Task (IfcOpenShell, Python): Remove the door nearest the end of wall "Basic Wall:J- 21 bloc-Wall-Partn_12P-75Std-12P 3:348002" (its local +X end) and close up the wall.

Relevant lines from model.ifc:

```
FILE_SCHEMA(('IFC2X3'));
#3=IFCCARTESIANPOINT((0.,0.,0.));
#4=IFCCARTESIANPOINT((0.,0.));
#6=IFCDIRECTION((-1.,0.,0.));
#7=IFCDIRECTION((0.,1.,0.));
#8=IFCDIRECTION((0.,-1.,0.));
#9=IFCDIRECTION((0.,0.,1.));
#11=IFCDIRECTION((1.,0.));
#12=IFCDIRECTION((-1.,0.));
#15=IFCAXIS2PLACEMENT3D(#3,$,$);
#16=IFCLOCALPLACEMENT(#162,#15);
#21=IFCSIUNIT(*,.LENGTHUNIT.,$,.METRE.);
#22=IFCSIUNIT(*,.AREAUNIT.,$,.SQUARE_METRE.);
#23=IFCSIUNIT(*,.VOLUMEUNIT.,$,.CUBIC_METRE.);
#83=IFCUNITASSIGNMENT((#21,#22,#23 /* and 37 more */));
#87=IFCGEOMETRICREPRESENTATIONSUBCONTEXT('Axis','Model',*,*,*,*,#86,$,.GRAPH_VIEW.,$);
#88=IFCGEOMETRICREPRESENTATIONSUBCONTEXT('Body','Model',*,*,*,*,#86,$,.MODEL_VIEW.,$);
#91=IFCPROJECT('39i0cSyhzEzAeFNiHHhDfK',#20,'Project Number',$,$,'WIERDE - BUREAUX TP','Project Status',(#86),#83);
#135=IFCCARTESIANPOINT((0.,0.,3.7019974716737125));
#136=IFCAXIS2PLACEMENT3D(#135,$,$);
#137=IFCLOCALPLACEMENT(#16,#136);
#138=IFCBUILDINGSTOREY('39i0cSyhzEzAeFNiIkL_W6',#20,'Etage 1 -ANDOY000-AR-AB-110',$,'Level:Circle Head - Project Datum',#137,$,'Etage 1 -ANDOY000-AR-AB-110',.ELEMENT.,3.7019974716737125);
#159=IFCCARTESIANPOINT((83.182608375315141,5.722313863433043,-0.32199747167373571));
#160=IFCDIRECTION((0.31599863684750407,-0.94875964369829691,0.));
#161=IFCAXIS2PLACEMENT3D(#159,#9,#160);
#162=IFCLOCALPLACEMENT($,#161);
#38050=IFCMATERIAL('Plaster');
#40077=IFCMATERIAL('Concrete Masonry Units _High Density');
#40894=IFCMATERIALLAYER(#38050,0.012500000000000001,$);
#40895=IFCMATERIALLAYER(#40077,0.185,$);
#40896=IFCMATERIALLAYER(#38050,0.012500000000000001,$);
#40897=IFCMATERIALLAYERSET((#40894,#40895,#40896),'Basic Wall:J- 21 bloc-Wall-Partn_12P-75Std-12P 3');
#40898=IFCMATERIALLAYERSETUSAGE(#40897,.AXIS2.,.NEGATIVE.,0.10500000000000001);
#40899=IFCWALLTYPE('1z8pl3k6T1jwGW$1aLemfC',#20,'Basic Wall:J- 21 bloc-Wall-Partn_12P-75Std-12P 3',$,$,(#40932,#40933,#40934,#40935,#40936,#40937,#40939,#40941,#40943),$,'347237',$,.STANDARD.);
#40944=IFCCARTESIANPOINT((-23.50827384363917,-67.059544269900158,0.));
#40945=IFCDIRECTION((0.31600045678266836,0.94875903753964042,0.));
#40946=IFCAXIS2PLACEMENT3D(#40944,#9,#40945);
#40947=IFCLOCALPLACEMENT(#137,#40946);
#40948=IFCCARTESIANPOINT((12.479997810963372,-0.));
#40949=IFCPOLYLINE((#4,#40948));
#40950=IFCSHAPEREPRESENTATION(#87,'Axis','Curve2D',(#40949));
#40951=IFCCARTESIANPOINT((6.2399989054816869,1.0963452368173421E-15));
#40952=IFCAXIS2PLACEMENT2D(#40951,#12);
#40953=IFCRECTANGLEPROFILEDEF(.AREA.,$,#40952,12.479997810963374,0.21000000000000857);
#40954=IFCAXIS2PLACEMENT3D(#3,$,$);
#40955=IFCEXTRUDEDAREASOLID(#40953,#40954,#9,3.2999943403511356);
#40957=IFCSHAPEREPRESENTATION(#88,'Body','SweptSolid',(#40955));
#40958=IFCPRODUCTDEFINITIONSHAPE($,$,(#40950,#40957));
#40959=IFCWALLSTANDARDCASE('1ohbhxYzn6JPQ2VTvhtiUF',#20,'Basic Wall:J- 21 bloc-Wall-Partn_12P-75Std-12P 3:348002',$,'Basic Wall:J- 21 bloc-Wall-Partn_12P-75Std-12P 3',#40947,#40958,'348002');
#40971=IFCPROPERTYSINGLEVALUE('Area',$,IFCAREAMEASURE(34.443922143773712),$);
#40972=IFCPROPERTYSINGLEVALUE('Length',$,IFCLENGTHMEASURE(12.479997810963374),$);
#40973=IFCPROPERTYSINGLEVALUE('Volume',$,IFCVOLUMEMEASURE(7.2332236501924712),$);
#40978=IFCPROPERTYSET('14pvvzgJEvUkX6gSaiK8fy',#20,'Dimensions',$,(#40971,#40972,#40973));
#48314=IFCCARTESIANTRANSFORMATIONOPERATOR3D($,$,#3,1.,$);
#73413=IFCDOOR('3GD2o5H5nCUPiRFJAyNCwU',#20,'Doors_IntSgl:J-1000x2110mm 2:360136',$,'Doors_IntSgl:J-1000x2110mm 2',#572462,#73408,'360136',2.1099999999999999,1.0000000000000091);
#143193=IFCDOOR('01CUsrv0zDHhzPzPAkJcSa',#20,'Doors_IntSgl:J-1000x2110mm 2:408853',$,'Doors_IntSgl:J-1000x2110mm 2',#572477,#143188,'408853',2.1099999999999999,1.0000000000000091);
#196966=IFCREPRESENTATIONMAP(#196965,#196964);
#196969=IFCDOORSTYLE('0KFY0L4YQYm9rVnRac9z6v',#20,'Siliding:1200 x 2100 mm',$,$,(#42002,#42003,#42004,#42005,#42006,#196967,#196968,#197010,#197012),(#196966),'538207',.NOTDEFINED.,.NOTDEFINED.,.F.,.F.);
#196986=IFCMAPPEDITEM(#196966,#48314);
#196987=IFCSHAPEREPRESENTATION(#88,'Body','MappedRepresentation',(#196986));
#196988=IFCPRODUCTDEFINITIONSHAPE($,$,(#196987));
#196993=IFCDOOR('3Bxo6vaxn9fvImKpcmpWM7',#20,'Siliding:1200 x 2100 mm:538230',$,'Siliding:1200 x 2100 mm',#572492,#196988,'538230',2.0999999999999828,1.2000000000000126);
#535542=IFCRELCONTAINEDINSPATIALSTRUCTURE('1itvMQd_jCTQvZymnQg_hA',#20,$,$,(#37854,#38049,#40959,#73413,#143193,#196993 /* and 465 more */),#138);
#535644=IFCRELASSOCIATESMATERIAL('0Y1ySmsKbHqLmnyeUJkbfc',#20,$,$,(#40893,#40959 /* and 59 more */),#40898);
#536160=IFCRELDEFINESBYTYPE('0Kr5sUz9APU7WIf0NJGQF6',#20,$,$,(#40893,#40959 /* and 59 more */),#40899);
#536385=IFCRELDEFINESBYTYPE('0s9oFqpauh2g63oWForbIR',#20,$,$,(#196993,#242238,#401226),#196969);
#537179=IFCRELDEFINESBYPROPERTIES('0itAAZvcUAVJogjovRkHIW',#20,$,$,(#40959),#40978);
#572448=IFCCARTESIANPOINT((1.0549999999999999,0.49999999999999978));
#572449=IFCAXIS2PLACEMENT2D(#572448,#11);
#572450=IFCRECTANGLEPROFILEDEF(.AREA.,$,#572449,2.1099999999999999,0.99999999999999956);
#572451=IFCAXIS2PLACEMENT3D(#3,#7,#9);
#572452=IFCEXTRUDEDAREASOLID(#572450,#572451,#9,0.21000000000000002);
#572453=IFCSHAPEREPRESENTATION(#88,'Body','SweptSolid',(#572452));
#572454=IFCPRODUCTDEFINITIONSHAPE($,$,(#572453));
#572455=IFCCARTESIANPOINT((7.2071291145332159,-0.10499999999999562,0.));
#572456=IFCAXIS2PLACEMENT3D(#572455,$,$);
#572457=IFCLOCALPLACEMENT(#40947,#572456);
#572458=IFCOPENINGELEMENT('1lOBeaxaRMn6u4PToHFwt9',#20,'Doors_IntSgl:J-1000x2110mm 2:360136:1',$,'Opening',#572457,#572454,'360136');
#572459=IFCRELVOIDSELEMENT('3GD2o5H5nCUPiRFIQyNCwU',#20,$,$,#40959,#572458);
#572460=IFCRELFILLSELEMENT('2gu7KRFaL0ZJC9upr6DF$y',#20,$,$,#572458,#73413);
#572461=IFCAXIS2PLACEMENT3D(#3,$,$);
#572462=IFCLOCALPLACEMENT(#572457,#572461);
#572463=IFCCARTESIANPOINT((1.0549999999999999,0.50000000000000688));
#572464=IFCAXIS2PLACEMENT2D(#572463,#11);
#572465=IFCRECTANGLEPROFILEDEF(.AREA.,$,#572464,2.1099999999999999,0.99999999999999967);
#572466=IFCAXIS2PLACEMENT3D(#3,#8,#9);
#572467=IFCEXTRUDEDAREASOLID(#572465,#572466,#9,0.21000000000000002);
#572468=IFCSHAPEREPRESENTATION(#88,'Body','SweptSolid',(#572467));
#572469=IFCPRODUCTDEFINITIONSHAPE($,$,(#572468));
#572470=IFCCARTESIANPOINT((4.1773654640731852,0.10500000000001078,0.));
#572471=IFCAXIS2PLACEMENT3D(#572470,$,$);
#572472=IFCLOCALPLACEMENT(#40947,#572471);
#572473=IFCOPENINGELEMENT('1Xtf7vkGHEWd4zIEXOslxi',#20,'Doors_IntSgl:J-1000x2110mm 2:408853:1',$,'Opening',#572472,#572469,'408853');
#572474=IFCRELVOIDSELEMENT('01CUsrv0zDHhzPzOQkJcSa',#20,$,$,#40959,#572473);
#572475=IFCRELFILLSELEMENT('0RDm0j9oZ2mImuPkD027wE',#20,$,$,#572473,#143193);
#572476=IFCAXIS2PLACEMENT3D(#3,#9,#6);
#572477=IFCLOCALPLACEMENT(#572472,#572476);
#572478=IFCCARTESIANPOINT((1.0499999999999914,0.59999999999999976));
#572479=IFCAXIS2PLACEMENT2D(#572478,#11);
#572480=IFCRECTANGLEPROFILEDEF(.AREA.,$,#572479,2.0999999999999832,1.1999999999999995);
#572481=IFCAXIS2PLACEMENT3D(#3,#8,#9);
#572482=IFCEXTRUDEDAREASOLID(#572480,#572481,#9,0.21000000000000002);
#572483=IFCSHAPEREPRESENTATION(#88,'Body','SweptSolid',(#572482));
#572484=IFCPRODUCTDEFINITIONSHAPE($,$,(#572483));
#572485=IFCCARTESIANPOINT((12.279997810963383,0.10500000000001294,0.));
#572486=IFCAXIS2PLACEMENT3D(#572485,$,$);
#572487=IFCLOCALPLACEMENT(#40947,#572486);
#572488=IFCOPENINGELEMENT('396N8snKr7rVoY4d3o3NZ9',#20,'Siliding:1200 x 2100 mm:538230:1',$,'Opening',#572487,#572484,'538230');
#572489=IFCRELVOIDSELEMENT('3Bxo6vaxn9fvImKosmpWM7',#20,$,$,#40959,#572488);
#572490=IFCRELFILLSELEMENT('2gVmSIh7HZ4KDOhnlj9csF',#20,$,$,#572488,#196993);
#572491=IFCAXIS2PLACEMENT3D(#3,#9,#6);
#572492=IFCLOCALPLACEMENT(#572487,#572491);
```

```python
import ifcopenshell
import ifcopenshell.api.feature
import ifcopenshell.api.pset
import ifcopenshell.api.root
import ifcopenshell.geom
import ifcopenshell.util.element
import ifcopenshell.util.shape
import ifcopenshell.util.unit

model = ifcopenshell.open("model.ifc")
area_scale = ifcopenshell.util.unit.calculate_unit_scale(model, "AREAUNIT")
volume_scale = ifcopenshell.util.unit.calculate_unit_scale(model, "VOLUMEUNIT")
settings = ifcopenshell.geom.settings()


def volume(element):
    """Net volume in cubic metres, openings subtracted."""
    shape = ifcopenshell.geom.create_shape(settings, element)
    return ifcopenshell.util.shape.get_volume(shape.geometry)


door = model.by_guid("3Bxo6vaxn9fvImKpcmpWM7")
opening = door.FillsVoids[0].RelatingOpeningElement
wall = opening.VoidsElements[0].RelatingBuildingElement
before = volume(wall)

ifcopenshell.api.root.remove_product(model, product=door)
ifcopenshell.api.feature.remove_feature(model, feature=opening)

after = volume(wall)
thickness = 0.21  # wall thickness in metres

# Update the wall's stored quantities.
pset = model.by_id(ifcopenshell.util.element.get_pset(wall, "Dimensions", should_inherit=False)["id"])
ifcopenshell.api.pset.edit_pset(model, pset=pset, properties={
    "Area": model.create_entity("IfcAreaMeasure", after / thickness / area_scale),
    "Volume": model.create_entity("IfcVolumeMeasure", after / volume_scale),
})

print(f"wall volume {before:.3f} -> {after:.3f} m3")

model.write("model_updated.ifc")
```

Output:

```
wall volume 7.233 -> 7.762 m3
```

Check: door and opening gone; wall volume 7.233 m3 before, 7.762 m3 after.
